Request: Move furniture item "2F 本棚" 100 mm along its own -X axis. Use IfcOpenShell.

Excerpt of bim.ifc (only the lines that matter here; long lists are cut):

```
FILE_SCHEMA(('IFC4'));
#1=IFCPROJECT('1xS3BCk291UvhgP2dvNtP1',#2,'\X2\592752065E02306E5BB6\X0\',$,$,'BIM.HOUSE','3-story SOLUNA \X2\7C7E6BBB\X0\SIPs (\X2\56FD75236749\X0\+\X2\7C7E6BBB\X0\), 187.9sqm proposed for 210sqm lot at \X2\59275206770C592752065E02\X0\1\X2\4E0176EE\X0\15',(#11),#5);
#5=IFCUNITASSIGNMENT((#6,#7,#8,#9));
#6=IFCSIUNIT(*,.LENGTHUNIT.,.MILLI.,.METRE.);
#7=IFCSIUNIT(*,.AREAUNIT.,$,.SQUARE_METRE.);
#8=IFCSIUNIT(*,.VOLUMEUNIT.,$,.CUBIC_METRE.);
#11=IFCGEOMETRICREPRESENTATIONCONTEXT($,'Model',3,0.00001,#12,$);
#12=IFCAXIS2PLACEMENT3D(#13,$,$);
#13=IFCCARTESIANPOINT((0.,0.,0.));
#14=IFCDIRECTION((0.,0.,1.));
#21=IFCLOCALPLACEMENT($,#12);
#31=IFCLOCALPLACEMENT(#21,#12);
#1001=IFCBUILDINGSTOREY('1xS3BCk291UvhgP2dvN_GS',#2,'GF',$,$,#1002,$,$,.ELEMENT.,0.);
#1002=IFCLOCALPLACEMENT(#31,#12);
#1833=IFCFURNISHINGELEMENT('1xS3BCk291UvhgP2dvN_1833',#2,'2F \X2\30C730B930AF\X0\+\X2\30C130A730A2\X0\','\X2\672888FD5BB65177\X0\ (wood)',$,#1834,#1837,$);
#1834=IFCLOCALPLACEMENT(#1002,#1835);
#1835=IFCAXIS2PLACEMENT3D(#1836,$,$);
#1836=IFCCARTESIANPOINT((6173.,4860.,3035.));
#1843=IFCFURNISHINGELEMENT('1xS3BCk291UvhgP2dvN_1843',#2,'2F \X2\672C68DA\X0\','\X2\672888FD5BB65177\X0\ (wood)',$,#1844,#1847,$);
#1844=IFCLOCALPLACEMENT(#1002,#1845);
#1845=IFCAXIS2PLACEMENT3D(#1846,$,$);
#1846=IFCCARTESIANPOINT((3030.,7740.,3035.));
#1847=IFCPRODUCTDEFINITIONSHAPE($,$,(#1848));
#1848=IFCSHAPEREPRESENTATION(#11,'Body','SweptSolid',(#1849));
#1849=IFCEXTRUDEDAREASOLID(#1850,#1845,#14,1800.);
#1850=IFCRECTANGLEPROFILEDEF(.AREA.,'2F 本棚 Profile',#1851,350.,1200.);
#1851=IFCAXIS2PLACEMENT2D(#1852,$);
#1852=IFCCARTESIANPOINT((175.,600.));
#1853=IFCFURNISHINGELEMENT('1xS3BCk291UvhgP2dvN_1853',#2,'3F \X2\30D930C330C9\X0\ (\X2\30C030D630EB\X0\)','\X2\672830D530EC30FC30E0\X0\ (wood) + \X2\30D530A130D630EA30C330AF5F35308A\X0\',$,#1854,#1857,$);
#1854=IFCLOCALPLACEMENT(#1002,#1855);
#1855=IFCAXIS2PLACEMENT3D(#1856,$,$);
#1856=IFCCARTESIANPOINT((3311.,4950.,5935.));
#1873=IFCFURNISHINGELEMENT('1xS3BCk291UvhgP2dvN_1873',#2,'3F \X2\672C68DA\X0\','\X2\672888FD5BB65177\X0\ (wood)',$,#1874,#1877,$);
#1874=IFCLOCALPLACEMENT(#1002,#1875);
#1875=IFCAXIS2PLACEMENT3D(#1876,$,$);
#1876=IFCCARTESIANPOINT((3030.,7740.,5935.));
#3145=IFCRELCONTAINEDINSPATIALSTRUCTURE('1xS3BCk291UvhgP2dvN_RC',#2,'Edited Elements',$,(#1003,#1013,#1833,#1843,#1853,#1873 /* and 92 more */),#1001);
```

```python
import ifcopenshell
import ifcopenshell.api.geometry
import ifcopenshell.util.placement

model = ifcopenshell.open("bim.ifc")

item = model.by_id(1843)
matrix = ifcopenshell.util.placement.get_local_placement(item.ObjectPlacement)
matrix[:3, 3] -= matrix[:3, 0] * 100.0
ifcopenshell.api.geometry.edit_object_placement(model, product=item, matrix=matrix, is_si=False)

print(ifcopenshell.util.placement.get_local_placement(item.ObjectPlacement).round(3) + 0.0)

model.write("bim_rev.ifc")
```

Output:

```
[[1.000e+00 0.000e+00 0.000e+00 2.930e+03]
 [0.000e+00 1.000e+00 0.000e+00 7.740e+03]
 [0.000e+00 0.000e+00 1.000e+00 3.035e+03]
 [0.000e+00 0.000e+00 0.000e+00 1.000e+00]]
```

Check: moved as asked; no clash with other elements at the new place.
